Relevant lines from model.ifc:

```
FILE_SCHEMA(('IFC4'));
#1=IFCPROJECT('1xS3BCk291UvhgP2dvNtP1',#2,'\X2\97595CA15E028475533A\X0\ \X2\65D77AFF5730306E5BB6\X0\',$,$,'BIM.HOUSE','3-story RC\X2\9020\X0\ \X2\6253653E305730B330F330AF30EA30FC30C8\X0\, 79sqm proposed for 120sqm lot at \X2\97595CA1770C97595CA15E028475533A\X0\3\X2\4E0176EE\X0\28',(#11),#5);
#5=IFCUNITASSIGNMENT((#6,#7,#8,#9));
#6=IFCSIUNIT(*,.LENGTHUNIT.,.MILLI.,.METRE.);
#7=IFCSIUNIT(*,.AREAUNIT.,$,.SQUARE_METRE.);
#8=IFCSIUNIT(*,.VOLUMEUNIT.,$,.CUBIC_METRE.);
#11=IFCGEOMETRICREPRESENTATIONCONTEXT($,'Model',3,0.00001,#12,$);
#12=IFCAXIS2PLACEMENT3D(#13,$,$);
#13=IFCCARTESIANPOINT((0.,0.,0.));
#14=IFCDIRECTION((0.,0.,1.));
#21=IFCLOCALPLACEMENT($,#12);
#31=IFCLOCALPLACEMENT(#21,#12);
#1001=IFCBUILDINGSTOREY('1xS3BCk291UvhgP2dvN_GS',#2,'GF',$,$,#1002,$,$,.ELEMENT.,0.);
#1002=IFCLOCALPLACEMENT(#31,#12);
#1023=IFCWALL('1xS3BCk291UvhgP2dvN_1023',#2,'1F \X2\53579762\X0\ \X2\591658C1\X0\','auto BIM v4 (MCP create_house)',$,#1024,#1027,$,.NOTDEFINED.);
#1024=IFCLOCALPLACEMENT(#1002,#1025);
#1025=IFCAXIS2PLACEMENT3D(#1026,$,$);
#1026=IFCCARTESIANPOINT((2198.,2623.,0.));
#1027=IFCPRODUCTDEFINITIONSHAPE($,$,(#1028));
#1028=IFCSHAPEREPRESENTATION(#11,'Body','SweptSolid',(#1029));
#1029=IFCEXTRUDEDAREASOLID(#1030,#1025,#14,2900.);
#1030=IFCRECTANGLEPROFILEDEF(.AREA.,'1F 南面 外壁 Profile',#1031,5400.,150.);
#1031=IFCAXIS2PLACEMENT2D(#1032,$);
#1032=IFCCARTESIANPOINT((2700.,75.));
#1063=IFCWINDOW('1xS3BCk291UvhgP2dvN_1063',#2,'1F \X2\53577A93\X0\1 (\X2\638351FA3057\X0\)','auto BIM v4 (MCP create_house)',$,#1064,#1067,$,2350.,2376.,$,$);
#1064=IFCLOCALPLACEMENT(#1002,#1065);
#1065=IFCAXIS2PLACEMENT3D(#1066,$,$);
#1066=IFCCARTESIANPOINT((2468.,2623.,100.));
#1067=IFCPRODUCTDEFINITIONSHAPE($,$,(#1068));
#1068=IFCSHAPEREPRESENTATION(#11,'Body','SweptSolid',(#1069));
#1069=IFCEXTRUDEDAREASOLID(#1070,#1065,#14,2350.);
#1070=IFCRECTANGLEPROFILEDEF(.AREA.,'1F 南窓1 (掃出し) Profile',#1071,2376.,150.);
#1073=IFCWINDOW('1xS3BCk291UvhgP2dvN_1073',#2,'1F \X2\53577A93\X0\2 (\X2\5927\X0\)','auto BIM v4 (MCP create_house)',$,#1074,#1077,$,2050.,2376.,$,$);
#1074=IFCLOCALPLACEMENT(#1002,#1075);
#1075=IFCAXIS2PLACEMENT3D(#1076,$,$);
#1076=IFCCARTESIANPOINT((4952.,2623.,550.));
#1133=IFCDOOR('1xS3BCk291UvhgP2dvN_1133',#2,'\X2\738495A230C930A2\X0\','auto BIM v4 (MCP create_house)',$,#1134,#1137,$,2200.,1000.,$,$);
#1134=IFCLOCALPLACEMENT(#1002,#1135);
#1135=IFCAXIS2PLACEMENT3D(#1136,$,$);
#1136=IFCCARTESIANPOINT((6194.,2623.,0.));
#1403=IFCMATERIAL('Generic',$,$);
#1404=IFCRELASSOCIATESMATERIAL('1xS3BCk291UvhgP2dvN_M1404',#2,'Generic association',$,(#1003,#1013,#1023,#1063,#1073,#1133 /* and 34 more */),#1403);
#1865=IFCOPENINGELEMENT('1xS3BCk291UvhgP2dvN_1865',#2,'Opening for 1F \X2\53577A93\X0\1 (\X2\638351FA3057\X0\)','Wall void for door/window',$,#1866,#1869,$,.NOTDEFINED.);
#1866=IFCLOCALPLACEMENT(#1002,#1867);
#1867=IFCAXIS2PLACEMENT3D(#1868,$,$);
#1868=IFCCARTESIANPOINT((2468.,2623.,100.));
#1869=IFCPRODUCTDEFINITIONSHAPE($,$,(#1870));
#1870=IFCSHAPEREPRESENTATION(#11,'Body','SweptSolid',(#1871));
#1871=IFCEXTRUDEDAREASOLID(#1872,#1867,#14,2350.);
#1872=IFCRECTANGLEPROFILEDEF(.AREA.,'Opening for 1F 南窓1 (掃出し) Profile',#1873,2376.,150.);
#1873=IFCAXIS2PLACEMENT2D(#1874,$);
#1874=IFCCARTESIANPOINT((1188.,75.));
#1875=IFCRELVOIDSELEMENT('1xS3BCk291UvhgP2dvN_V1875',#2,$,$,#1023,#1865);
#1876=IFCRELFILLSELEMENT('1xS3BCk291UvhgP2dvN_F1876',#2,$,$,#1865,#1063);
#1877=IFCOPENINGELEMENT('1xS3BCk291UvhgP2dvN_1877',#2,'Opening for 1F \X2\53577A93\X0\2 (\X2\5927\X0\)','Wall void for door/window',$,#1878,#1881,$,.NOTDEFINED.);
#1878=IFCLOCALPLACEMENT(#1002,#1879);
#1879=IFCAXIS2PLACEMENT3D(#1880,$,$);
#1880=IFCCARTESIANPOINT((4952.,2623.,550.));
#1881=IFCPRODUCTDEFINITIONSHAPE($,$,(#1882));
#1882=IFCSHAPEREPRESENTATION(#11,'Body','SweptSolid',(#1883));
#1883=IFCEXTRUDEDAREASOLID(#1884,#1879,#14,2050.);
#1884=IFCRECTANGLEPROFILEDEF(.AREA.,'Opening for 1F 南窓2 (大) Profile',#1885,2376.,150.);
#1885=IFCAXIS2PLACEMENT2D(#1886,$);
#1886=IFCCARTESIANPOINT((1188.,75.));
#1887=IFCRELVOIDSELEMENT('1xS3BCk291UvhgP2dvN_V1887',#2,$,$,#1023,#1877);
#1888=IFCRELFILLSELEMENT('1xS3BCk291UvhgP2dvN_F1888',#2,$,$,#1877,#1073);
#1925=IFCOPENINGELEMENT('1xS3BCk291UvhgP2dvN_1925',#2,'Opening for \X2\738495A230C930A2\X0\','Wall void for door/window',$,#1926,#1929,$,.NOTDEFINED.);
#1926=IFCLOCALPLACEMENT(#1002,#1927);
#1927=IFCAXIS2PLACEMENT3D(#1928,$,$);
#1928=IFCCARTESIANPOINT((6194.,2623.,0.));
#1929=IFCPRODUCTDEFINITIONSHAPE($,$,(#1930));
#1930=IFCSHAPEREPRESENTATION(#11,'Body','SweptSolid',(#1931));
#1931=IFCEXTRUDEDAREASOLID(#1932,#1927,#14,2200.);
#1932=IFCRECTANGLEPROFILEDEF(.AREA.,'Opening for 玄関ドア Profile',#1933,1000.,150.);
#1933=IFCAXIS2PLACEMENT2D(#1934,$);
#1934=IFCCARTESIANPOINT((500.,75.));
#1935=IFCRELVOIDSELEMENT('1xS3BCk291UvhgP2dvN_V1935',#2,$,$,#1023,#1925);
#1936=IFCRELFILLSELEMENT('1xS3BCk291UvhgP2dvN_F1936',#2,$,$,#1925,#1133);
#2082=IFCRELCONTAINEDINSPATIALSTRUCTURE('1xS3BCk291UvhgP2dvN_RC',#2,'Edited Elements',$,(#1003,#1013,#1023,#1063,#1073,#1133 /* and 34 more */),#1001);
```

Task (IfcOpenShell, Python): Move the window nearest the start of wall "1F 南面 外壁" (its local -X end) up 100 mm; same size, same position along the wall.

```python
import numpy as np
import ifcopenshell
import ifcopenshell.api.geometry
import ifcopenshell.util.placement
import ifcopenshell.util.unit

model = ifcopenshell.open("model.ifc")
unit_scale = ifcopenshell.util.unit.calculate_unit_scale(model)

window = model.by_guid("1xS3BCk291UvhgP2dvN_1063")
opening = window.FillsVoids[0].RelatingOpeningElement
dz = 100.0

shift = np.array([0.0, 0.0, dz])
# The window is not placed relative to its opening, so move both.
for product in (opening, window):
    matrix = ifcopenshell.util.placement.get_local_placement(product.ObjectPlacement)
    matrix[:3, 3] += shift
    ifcopenshell.api.geometry.edit_object_placement(model, product=product, matrix=matrix, is_si=False)

print(f"moved by {dz * unit_scale:+.3f} m")

model.write("model_rev.ifc")
```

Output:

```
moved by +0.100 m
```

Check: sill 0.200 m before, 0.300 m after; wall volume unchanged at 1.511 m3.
